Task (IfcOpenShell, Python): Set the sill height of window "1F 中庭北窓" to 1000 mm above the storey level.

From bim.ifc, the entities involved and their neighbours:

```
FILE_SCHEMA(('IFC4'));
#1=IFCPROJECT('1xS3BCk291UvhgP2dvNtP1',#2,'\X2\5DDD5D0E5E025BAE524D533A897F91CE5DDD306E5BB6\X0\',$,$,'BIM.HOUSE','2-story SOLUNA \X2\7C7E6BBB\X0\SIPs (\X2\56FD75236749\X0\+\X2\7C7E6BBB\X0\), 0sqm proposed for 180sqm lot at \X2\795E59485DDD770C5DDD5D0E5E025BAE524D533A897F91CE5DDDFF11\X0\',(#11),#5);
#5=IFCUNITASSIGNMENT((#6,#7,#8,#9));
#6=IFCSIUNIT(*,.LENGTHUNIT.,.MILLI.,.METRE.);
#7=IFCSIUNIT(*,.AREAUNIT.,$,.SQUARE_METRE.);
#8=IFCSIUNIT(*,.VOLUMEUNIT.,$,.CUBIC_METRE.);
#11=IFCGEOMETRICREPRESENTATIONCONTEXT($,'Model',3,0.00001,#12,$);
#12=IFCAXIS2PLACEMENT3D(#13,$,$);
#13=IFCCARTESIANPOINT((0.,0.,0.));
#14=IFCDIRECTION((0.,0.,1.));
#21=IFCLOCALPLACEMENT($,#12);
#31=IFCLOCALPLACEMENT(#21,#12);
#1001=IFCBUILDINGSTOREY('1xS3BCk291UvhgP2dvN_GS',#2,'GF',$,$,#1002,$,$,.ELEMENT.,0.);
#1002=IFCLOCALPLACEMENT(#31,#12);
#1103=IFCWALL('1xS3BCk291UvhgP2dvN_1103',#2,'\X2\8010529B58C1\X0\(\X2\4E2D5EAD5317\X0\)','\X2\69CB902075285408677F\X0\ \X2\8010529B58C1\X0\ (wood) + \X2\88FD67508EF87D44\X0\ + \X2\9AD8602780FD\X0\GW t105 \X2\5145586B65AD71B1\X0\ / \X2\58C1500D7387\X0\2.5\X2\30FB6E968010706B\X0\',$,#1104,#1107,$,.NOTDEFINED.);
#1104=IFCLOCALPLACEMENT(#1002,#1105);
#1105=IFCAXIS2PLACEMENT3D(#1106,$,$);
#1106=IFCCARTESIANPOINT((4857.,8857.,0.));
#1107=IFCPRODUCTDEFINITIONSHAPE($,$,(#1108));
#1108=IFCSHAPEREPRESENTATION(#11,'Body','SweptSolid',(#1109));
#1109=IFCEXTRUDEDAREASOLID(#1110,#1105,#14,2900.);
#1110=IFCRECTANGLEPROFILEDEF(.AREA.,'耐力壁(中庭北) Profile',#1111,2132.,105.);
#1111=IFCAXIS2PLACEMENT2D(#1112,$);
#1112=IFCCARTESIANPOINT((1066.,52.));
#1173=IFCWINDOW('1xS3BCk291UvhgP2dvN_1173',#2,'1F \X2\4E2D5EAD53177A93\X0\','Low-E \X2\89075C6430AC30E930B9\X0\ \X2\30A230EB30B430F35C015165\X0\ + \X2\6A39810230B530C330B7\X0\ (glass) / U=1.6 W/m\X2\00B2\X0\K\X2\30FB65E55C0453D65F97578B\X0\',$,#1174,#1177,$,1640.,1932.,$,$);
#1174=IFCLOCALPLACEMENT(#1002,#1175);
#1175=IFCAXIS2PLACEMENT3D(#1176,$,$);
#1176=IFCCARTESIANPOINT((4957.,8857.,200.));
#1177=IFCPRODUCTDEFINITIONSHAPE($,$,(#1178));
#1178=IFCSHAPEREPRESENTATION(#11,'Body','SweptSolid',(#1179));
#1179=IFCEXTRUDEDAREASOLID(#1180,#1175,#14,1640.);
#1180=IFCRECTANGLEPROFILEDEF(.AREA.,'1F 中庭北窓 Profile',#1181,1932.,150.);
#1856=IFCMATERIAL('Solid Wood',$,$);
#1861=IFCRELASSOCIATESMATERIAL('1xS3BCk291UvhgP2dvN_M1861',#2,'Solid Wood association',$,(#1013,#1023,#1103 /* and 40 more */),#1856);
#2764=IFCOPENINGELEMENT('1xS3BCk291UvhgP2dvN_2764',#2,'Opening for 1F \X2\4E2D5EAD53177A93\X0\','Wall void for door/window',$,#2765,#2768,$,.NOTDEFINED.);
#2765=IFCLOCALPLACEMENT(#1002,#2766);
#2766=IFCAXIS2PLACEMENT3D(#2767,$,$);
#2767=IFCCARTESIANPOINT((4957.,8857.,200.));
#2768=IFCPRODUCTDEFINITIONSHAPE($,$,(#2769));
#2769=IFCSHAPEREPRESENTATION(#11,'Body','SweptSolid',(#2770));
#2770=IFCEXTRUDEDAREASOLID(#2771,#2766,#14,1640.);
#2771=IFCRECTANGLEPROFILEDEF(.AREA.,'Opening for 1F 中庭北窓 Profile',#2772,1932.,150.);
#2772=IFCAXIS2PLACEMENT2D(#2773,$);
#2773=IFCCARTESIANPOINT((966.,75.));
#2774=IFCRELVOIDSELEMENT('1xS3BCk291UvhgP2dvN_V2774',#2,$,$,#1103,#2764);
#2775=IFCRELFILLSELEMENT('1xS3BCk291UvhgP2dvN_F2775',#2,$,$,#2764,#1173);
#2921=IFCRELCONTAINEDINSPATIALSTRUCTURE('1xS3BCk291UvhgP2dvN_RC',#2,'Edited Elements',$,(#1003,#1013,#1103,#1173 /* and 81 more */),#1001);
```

```python
import numpy as np
import ifcopenshell
import ifcopenshell.api.geometry
import ifcopenshell.geom
import ifcopenshell.util.element
import ifcopenshell.util.placement
import ifcopenshell.util.shape
import ifcopenshell.util.unit

model = ifcopenshell.open("bim.ifc")
unit_scale = ifcopenshell.util.unit.calculate_unit_scale(model)

window = model.by_guid("1xS3BCk291UvhgP2dvN_1173")
opening = window.FillsVoids[0].RelatingOpeningElement
storey = ifcopenshell.util.element.get_container(window, ifc_class="IfcBuildingStorey")
level = ifcopenshell.util.placement.get_local_placement(storey.ObjectPlacement)[2, 3]

# The opening's origin need not be at the sill, so measure its lowest point.
shape = ifcopenshell.geom.create_shape(ifcopenshell.geom.settings(), opening)
bottom = ifcopenshell.util.shape.get_shape_bottom_elevation(shape, shape.geometry) / unit_scale
dz = level + 1000.0 - bottom

shift = np.array([0.0, 0.0, dz])
# The window is not placed relative to its opening, so move both.
for product in (opening, window):
    matrix = ifcopenshell.util.placement.get_local_placement(product.ObjectPlacement)
    matrix[:3, 3] += shift
    ifcopenshell.api.geometry.edit_object_placement(model, product=product, matrix=matrix, is_si=False)

print(f"moved by {dz * unit_scale:+.3f} m")

model.write("bim_v2.ifc")
```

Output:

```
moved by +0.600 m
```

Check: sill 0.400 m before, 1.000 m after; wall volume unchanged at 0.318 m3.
